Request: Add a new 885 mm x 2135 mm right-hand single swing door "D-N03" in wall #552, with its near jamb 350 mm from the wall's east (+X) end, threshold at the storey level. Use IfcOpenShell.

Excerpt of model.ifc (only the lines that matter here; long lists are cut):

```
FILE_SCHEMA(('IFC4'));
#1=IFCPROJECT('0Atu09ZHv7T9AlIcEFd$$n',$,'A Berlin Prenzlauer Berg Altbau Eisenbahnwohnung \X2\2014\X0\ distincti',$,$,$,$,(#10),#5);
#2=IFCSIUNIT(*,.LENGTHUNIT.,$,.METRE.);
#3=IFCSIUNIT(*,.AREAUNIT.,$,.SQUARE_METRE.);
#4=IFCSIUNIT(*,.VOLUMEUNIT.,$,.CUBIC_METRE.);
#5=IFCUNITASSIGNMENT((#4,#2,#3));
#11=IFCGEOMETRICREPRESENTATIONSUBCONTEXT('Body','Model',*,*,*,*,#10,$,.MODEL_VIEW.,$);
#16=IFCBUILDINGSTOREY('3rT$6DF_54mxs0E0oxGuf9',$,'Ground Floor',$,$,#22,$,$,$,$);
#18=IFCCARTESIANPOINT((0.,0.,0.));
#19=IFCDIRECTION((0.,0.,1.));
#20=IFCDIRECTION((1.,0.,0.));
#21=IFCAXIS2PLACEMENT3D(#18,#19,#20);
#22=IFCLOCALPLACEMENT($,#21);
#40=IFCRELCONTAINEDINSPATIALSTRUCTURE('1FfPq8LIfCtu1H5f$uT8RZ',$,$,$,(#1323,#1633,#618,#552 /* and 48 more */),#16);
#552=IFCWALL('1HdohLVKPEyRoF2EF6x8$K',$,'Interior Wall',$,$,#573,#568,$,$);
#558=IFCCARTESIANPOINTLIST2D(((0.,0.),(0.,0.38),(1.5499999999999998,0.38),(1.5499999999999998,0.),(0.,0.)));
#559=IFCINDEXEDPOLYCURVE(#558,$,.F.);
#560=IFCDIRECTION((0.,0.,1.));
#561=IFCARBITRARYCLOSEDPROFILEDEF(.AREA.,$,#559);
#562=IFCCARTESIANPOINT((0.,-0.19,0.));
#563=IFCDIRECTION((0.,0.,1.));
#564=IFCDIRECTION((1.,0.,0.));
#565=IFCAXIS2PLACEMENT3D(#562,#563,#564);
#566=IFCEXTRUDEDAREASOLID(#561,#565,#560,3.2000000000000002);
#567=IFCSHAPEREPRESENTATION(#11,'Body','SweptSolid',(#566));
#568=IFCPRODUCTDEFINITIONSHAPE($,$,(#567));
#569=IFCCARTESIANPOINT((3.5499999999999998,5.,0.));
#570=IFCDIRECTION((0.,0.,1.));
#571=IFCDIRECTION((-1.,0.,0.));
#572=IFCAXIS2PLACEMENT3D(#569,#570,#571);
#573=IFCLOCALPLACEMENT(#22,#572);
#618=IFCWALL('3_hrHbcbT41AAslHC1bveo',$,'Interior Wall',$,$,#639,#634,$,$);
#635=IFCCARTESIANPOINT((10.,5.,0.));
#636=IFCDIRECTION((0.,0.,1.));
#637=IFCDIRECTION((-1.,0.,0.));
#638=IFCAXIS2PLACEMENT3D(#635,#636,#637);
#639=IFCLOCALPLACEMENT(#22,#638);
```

```python
import numpy as np
import ifcopenshell
import ifcopenshell.api.feature
import ifcopenshell.api.geometry
import ifcopenshell.api.root
import ifcopenshell.api.spatial
import ifcopenshell.geom
import ifcopenshell.util.element
import ifcopenshell.util.placement
import ifcopenshell.util.representation
import ifcopenshell.util.shape
import ifcopenshell.util.unit

model = ifcopenshell.open("model.ifc")
unit_scale = ifcopenshell.util.unit.calculate_unit_scale(model)
settings = ifcopenshell.geom.settings()


def volume(element):
    """Net volume in cubic metres, openings subtracted."""
    shape = ifcopenshell.geom.create_shape(settings, element)
    return ifcopenshell.util.shape.get_volume(shape.geometry)


wall = model.by_id(552)
storey = ifcopenshell.util.element.get_container(wall, ifc_class="IfcBuildingStorey")
context = ifcopenshell.util.representation.get_context(model, "Model", "Body", "MODEL_VIEW")
before = volume(wall)

width, height, from_end, sill = 0.885, 2.135, 0.35, 0.0  # metres

# The wall runs along its own X axis, and the end named is its -X end.
wall_shape = ifcopenshell.geom.create_shape(settings, wall)
x, y, z = ifcopenshell.util.shape.get_vertices(wall_shape.geometry).T
start = x.min() + from_end
face, thickness = float(y.min()), float(y.max() - y.min())
wall_matrix = ifcopenshell.util.placement.get_local_placement(wall.ObjectPlacement)
level = ifcopenshell.util.placement.get_local_placement(storey.ObjectPlacement)[2, 3]


def in_wall(x, y):
    """Placement at x, y metres in the wall's axes, at sill height."""
    matrix = wall_matrix.copy()
    matrix[:, 3] = wall_matrix @ np.array([x / unit_scale, y / unit_scale, 0.0, 1.0])
    matrix[2, 3] = level + sill / unit_scale
    return matrix


# Opening: a box that overshoots both wall faces by 50 mm.
opening = ifcopenshell.api.root.create_entity(model, ifc_class="IfcOpeningElement", predefined_type="OPENING")
box = ifcopenshell.api.geometry.add_wall_representation(
    model, context=context, length=width, height=height, thickness=thickness + 0.1
)
ifcopenshell.api.geometry.assign_representation(model, product=opening, representation=box)
ifcopenshell.api.geometry.edit_object_placement(model, product=opening, matrix=in_wall(start, face - 0.05), is_si=False)
ifcopenshell.api.feature.add_feature(model, feature=opening, element=wall)

door = ifcopenshell.api.root.create_entity(model, ifc_class="IfcDoor", name="D-N03", predefined_type="DOOR")
door.OverallWidth, door.OverallHeight = width / unit_scale, height / unit_scale
door.OperationType = "SINGLE_SWING_RIGHT"
body = ifcopenshell.api.geometry.add_door_representation(
    model,
    context=context,
    overall_width=door.OverallWidth,
    overall_height=door.OverallHeight,
    operation_type="SINGLE_SWING_RIGHT",
    lining_properties={"LiningDepth": thickness / unit_scale, "ThresholdDepth": thickness / unit_scale},
)
ifcopenshell.api.geometry.assign_representation(model, product=door, representation=body)
ifcopenshell.api.spatial.assign_container(model, products=[door], relating_structure=storey)
ifcopenshell.api.feature.add_filling(model, opening=opening, element=door)

# The lining spans the wall, so the door starts at the wall face.
ifcopenshell.api.geometry.edit_object_placement(model, product=door, matrix=in_wall(start, face), is_si=False)

after = volume(wall)

print(f"wall volume {before:.3f} -> {after:.3f} m3")

model.write("model_edited.ifc")
```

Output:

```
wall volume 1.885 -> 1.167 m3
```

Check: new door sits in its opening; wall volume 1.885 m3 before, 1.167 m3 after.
